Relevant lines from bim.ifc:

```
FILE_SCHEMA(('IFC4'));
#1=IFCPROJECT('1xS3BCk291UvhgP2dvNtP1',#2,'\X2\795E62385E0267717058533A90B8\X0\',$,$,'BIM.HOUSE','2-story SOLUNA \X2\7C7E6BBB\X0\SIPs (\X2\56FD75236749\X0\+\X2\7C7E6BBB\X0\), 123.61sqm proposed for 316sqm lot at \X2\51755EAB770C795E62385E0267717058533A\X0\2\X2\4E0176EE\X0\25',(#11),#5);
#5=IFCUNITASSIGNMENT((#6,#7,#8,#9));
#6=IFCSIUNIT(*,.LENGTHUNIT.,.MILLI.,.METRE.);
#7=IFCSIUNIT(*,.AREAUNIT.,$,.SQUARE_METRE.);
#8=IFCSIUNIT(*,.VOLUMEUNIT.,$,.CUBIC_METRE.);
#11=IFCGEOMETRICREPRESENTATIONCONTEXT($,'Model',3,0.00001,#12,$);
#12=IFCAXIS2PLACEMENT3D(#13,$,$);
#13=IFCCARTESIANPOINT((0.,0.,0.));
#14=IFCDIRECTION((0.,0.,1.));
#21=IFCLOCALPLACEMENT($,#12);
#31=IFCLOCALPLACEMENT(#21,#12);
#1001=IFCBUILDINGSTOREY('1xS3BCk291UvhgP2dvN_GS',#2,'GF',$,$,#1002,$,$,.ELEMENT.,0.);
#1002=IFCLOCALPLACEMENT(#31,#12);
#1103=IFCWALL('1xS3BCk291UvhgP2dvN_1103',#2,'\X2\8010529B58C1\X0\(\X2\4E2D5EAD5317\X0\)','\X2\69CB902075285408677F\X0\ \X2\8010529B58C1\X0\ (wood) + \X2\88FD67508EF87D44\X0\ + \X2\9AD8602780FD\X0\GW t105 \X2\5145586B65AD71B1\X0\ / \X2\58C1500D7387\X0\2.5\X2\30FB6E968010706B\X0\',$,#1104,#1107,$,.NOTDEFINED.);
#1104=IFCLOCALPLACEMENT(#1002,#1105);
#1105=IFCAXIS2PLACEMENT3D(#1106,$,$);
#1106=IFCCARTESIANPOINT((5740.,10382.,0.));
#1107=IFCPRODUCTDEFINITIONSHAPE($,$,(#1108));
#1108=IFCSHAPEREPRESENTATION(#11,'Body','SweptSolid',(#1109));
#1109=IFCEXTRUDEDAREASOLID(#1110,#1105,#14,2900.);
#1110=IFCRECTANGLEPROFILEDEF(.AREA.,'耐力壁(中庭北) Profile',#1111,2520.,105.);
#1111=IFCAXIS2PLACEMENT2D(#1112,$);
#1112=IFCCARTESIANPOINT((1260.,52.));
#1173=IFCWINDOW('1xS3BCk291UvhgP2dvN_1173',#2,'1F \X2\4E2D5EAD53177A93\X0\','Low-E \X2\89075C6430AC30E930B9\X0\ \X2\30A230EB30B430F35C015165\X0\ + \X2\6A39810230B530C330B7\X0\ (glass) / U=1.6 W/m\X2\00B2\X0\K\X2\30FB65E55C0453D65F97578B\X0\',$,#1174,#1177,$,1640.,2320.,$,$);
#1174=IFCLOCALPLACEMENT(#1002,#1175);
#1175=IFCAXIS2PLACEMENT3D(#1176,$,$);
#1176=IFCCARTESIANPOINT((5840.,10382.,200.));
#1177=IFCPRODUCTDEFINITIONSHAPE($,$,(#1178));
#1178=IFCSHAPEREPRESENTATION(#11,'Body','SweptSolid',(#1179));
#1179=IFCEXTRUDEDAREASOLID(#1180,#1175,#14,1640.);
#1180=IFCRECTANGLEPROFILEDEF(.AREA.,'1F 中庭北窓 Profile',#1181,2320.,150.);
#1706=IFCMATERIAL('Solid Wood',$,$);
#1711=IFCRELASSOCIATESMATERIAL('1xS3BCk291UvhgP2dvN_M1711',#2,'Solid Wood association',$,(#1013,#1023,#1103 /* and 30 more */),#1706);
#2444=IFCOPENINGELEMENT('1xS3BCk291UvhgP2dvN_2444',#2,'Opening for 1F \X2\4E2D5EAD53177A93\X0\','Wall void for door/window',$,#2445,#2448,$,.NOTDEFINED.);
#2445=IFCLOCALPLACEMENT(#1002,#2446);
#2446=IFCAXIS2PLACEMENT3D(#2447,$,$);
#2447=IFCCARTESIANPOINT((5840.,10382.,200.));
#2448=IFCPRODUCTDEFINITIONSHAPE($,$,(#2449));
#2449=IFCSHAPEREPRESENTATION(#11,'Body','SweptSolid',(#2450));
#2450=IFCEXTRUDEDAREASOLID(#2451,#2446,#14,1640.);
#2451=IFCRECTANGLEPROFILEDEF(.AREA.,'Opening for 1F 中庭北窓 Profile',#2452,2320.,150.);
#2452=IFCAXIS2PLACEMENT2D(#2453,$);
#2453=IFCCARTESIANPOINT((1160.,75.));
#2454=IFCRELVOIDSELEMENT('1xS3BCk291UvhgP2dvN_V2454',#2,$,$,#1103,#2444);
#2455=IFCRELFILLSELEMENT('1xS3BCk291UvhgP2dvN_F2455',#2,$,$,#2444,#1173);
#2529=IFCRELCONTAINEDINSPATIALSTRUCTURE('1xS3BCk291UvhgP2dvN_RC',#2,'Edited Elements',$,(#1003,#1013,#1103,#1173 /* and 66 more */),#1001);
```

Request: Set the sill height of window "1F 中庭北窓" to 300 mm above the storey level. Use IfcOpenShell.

```python
import numpy as np
import ifcopenshell
import ifcopenshell.api.geometry
import ifcopenshell.geom
import ifcopenshell.util.element
import ifcopenshell.util.placement
import ifcopenshell.util.shape
import ifcopenshell.util.unit

model = ifcopenshell.open("bim.ifc")
unit_scale = ifcopenshell.util.unit.calculate_unit_scale(model)

window = model.by_guid("1xS3BCk291UvhgP2dvN_1173")
opening = window.FillsVoids[0].RelatingOpeningElement
storey = ifcopenshell.util.element.get_container(window, ifc_class="IfcBuildingStorey")
level = ifcopenshell.util.placement.get_local_placement(storey.ObjectPlacement)[2, 3]

# The opening's origin need not be at the sill, so measure its lowest point.
shape = ifcopenshell.geom.create_shape(ifcopenshell.geom.settings(), opening)
bottom = ifcopenshell.util.shape.get_shape_bottom_elevation(shape, shape.geometry) / unit_scale
dz = level + 300.0 - bottom

shift = np.array([0.0, 0.0, dz])
# The window is not placed relative to its opening, so move both.
for product in (opening, window):
    matrix = ifcopenshell.util.placement.get_local_placement(product.ObjectPlacement)
    matrix[:3, 3] += shift
    ifcopenshell.api.geometry.edit_object_placement(model, product=product, matrix=matrix, is_si=False)

print(f"moved by {dz * unit_scale:+.3f} m")

model.write("bim_updated.ifc")
```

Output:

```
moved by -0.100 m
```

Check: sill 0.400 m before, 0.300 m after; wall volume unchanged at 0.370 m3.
